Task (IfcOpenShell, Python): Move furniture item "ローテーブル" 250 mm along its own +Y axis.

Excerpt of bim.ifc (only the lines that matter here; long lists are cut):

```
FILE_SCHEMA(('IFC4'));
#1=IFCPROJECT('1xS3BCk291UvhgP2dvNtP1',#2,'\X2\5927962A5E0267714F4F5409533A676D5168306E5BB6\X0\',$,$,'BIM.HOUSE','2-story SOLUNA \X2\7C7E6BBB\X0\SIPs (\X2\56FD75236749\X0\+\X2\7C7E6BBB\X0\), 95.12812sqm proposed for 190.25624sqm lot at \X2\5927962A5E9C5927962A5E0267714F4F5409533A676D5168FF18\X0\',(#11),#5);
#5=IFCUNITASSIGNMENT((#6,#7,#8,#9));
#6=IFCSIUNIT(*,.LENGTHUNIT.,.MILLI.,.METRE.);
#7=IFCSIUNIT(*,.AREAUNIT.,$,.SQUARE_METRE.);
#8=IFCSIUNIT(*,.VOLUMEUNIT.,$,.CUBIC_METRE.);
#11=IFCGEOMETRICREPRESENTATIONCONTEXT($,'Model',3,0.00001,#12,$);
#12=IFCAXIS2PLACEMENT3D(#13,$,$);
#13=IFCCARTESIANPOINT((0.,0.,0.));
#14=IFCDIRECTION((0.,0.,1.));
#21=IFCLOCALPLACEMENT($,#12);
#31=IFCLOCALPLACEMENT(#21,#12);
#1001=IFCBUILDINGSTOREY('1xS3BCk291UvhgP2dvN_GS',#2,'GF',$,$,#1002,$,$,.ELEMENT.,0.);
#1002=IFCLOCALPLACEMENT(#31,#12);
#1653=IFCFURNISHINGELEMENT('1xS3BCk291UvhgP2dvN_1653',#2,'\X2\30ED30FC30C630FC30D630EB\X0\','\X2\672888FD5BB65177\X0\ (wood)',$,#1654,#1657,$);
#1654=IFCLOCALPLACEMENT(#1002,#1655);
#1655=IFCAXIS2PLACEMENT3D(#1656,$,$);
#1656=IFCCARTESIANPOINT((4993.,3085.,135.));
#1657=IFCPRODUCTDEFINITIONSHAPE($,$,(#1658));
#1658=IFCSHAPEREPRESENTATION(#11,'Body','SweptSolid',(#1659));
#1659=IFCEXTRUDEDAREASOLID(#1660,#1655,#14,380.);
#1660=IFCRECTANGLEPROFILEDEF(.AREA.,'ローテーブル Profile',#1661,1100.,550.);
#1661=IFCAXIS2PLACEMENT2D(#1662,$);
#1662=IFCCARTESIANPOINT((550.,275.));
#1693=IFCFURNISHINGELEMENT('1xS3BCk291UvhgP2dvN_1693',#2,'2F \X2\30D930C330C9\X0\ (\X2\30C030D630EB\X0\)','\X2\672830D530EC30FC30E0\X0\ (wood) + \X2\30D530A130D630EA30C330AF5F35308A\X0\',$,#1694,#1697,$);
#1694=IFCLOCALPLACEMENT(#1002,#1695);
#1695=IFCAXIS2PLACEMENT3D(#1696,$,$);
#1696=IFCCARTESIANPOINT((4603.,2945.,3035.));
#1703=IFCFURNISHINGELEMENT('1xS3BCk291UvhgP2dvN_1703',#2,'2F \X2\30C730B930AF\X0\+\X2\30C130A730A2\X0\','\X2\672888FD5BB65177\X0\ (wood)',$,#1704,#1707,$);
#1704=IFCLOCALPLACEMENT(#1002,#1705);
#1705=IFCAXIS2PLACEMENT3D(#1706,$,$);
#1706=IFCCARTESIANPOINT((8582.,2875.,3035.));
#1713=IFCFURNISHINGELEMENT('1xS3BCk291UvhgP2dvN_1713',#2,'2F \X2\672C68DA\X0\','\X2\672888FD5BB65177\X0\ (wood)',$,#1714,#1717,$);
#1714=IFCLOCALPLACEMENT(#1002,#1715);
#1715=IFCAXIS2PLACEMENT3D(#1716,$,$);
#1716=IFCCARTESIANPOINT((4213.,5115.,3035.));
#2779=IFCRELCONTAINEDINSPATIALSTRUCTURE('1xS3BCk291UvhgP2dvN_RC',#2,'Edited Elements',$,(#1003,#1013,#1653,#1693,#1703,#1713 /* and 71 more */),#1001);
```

```python
import ifcopenshell
import ifcopenshell.api.geometry
import ifcopenshell.util.placement

model = ifcopenshell.open("bim.ifc")

item = model.by_id(1653)
matrix = ifcopenshell.util.placement.get_local_placement(item.ObjectPlacement)
matrix[:3, 3] += matrix[:3, 1] * 250.0
ifcopenshell.api.geometry.edit_object_placement(model, product=item, matrix=matrix, is_si=False)

print(ifcopenshell.util.placement.get_local_placement(item.ObjectPlacement).round(3) + 0.0)

model.write("bim-out.ifc")
```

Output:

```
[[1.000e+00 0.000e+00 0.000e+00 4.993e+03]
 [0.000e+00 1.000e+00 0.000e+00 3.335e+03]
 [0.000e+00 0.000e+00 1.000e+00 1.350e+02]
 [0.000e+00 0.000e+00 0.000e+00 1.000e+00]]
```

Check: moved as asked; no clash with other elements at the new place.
